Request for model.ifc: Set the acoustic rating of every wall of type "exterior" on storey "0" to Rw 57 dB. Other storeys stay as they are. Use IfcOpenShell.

First a look at what the model holds.

```python
import ifcopenshell
import ifcopenshell.util.element

model = ifcopenshell.open("model.ifc")
print(model.schema)
storey = next(s for s in model.by_type("IfcBuildingStorey") if s.Name == "0")
walls = [e for e in ifcopenshell.util.element.get_decomposition(storey) if e.is_a("IfcWall")]
seen = {}
for e in walls:
    element_type = ifcopenshell.util.element.get_type(e)
    key = (element_type.Name if element_type != e and element_type else None, ifcopenshell.util.element.get_pset(e, "Pset_WallCommon", "AcousticRating"))
    seen[key] = seen.get(key, 0) + 1
for (name, value), count in sorted(seen.items(), key=str):
    print(count, "x", name, "|", value)
```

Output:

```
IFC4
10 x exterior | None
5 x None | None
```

```python
import ifcopenshell
import ifcopenshell.api.pset
import ifcopenshell.util.element

model = ifcopenshell.open("model.ifc")

storey = next(s for s in model.by_type("IfcBuildingStorey") if s.Name == "0")
walls = [e for e in ifcopenshell.util.element.get_decomposition(storey) if e.is_a("IfcWall")]

count = 0
for e in walls:
    element_type = ifcopenshell.util.element.get_type(e)
    if element_type in (None, e) or element_type.Name != "exterior":
        continue
    # add_pset returns the element's existing set when there is one.
    pset = ifcopenshell.api.pset.add_pset(model, product=e, name="Pset_WallCommon")
    ifcopenshell.api.pset.edit_pset(model, pset=pset, properties={"AcousticRating": "Rw 57 dB"})
    count += 1

print(count, "walls updated")

model.write("model_v2.ifc")
```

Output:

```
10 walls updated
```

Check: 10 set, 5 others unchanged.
